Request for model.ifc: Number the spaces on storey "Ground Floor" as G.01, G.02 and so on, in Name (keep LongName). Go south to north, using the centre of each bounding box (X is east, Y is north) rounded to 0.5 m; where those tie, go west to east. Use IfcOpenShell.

First a look at what the model holds.

```python
import ifcopenshell
import ifcopenshell.util.element
import ifcopenshell.util.placement

model = ifcopenshell.open("model.ifc")
print(model.schema)
storey = next(s for s in model.by_type("IfcBuildingStorey") if s.Name == "Ground Floor")
spaces = [e for e in ifcopenshell.util.element.get_decomposition(storey) if e.is_a("IfcSpace")]
for e in sorted(spaces, key=lambda e: e.id()):
    origin = ifcopenshell.util.placement.get_local_placement(e.ObjectPlacement)[:3, 3]
    print(e.id(), e.Name, e.LongName, origin.round(2) + 0.0, sep=" | ")
```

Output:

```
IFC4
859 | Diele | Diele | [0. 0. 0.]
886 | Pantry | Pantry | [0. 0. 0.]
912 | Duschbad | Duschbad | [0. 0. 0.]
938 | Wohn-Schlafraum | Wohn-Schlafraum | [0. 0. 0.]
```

```python
import ifcopenshell
import ifcopenshell.geom
import ifcopenshell.util.element
import ifcopenshell.util.shape

model = ifcopenshell.open("model.ifc")
settings = ifcopenshell.geom.settings()
settings.set("use-world-coords", True)


def centre(element):
    shape = ifcopenshell.geom.create_shape(settings, element)
    return ifcopenshell.util.shape.get_bbox_centroid(shape.geometry)


storey = next(s for s in model.by_type("IfcBuildingStorey") if s.Name == "Ground Floor")
spaces = [e for e in ifcopenshell.util.element.get_decomposition(storey) if e.is_a("IfcSpace")]

# Insertion points can sit at a corner or the storey origin, so sort by the geometry (in metres).
centres = {e: centre(e) for e in spaces}
spaces.sort(key=lambda e: (round(centres[e][1] / 0.5), centres[e][0]))

for i, e in enumerate(spaces, start=1):
    number = f"G.{i:02d}"
    e.Name = number
    print(e.id(), number)

model.write("model_v2.ifc")
```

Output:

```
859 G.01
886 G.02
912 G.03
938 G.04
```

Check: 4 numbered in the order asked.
